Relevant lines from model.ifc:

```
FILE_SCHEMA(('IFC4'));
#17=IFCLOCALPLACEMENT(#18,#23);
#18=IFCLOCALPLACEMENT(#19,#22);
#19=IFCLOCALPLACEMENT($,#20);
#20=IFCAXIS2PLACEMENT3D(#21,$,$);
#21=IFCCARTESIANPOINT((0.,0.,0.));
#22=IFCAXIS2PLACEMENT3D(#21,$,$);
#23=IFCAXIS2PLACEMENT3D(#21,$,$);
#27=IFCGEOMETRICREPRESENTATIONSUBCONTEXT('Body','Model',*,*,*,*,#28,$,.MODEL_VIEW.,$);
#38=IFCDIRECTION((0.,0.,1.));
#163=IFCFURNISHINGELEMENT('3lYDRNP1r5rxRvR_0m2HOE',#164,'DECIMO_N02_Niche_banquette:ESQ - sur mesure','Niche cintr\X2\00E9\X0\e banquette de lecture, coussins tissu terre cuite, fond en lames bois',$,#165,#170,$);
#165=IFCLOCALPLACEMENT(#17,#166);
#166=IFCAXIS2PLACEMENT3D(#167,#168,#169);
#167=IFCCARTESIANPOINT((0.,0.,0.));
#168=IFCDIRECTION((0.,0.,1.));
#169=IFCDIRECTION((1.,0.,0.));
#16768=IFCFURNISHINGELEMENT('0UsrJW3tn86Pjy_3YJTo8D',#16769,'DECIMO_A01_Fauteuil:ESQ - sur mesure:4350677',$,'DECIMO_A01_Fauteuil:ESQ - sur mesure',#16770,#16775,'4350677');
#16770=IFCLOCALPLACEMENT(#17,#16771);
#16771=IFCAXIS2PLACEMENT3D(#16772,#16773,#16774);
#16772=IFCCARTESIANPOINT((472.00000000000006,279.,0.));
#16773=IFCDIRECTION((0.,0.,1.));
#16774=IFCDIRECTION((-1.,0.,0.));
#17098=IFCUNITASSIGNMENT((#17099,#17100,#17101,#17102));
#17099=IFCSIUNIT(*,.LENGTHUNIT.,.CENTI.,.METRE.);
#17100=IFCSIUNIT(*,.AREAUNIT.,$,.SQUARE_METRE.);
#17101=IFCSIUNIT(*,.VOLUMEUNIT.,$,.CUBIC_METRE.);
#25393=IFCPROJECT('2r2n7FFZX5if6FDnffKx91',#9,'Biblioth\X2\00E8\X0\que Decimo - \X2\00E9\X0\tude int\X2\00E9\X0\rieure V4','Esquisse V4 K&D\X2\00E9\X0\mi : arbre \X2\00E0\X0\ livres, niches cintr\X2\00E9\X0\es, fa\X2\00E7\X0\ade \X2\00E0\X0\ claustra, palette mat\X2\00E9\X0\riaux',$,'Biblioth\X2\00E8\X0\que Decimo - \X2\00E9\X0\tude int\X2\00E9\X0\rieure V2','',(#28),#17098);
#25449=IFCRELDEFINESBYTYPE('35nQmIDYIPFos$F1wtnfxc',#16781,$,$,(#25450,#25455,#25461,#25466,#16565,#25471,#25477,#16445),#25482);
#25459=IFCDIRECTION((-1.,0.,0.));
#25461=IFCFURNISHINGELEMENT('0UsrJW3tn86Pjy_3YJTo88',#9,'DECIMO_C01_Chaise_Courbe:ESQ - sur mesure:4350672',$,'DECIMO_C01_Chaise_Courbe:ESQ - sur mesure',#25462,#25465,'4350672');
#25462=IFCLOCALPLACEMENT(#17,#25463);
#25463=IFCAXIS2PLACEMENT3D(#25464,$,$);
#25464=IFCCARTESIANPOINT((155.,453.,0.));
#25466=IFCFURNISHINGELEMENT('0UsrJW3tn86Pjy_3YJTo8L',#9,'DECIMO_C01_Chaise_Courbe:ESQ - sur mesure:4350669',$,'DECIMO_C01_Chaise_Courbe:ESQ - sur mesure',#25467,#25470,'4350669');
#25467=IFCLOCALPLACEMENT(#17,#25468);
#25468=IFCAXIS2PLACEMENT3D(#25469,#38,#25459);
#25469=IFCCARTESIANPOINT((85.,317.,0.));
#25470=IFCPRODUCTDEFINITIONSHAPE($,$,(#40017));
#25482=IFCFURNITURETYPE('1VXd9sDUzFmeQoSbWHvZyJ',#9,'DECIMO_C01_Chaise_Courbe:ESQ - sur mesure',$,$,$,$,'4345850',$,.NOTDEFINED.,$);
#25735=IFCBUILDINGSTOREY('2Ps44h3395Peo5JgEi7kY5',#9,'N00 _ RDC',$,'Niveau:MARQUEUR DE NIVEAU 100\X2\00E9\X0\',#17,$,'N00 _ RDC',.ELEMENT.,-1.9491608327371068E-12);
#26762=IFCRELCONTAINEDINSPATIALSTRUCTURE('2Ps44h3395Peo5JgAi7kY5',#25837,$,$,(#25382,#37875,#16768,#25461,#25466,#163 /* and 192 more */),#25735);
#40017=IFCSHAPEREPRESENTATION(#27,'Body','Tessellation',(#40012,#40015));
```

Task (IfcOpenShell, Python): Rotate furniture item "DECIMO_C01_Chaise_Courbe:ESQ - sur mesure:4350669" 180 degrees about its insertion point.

```python
import ifcopenshell
import ifcopenshell.api.geometry
import ifcopenshell.util.placement

model = ifcopenshell.open("model.ifc")

item = model.by_guid("0UsrJW3tn86Pjy_3YJTo8L")
matrix = ifcopenshell.util.placement.get_local_placement(item.ObjectPlacement)
matrix = matrix @ ifcopenshell.util.placement.rotation(180, "Z")
ifcopenshell.api.geometry.edit_object_placement(model, product=item, matrix=matrix, is_si=False)

print(ifcopenshell.util.placement.get_local_placement(item.ObjectPlacement).round(3) + 0.0)

model.write("model_rev.ifc")
```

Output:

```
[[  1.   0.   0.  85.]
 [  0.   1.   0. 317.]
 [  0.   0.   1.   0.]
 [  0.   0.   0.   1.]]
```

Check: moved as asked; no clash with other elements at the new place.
